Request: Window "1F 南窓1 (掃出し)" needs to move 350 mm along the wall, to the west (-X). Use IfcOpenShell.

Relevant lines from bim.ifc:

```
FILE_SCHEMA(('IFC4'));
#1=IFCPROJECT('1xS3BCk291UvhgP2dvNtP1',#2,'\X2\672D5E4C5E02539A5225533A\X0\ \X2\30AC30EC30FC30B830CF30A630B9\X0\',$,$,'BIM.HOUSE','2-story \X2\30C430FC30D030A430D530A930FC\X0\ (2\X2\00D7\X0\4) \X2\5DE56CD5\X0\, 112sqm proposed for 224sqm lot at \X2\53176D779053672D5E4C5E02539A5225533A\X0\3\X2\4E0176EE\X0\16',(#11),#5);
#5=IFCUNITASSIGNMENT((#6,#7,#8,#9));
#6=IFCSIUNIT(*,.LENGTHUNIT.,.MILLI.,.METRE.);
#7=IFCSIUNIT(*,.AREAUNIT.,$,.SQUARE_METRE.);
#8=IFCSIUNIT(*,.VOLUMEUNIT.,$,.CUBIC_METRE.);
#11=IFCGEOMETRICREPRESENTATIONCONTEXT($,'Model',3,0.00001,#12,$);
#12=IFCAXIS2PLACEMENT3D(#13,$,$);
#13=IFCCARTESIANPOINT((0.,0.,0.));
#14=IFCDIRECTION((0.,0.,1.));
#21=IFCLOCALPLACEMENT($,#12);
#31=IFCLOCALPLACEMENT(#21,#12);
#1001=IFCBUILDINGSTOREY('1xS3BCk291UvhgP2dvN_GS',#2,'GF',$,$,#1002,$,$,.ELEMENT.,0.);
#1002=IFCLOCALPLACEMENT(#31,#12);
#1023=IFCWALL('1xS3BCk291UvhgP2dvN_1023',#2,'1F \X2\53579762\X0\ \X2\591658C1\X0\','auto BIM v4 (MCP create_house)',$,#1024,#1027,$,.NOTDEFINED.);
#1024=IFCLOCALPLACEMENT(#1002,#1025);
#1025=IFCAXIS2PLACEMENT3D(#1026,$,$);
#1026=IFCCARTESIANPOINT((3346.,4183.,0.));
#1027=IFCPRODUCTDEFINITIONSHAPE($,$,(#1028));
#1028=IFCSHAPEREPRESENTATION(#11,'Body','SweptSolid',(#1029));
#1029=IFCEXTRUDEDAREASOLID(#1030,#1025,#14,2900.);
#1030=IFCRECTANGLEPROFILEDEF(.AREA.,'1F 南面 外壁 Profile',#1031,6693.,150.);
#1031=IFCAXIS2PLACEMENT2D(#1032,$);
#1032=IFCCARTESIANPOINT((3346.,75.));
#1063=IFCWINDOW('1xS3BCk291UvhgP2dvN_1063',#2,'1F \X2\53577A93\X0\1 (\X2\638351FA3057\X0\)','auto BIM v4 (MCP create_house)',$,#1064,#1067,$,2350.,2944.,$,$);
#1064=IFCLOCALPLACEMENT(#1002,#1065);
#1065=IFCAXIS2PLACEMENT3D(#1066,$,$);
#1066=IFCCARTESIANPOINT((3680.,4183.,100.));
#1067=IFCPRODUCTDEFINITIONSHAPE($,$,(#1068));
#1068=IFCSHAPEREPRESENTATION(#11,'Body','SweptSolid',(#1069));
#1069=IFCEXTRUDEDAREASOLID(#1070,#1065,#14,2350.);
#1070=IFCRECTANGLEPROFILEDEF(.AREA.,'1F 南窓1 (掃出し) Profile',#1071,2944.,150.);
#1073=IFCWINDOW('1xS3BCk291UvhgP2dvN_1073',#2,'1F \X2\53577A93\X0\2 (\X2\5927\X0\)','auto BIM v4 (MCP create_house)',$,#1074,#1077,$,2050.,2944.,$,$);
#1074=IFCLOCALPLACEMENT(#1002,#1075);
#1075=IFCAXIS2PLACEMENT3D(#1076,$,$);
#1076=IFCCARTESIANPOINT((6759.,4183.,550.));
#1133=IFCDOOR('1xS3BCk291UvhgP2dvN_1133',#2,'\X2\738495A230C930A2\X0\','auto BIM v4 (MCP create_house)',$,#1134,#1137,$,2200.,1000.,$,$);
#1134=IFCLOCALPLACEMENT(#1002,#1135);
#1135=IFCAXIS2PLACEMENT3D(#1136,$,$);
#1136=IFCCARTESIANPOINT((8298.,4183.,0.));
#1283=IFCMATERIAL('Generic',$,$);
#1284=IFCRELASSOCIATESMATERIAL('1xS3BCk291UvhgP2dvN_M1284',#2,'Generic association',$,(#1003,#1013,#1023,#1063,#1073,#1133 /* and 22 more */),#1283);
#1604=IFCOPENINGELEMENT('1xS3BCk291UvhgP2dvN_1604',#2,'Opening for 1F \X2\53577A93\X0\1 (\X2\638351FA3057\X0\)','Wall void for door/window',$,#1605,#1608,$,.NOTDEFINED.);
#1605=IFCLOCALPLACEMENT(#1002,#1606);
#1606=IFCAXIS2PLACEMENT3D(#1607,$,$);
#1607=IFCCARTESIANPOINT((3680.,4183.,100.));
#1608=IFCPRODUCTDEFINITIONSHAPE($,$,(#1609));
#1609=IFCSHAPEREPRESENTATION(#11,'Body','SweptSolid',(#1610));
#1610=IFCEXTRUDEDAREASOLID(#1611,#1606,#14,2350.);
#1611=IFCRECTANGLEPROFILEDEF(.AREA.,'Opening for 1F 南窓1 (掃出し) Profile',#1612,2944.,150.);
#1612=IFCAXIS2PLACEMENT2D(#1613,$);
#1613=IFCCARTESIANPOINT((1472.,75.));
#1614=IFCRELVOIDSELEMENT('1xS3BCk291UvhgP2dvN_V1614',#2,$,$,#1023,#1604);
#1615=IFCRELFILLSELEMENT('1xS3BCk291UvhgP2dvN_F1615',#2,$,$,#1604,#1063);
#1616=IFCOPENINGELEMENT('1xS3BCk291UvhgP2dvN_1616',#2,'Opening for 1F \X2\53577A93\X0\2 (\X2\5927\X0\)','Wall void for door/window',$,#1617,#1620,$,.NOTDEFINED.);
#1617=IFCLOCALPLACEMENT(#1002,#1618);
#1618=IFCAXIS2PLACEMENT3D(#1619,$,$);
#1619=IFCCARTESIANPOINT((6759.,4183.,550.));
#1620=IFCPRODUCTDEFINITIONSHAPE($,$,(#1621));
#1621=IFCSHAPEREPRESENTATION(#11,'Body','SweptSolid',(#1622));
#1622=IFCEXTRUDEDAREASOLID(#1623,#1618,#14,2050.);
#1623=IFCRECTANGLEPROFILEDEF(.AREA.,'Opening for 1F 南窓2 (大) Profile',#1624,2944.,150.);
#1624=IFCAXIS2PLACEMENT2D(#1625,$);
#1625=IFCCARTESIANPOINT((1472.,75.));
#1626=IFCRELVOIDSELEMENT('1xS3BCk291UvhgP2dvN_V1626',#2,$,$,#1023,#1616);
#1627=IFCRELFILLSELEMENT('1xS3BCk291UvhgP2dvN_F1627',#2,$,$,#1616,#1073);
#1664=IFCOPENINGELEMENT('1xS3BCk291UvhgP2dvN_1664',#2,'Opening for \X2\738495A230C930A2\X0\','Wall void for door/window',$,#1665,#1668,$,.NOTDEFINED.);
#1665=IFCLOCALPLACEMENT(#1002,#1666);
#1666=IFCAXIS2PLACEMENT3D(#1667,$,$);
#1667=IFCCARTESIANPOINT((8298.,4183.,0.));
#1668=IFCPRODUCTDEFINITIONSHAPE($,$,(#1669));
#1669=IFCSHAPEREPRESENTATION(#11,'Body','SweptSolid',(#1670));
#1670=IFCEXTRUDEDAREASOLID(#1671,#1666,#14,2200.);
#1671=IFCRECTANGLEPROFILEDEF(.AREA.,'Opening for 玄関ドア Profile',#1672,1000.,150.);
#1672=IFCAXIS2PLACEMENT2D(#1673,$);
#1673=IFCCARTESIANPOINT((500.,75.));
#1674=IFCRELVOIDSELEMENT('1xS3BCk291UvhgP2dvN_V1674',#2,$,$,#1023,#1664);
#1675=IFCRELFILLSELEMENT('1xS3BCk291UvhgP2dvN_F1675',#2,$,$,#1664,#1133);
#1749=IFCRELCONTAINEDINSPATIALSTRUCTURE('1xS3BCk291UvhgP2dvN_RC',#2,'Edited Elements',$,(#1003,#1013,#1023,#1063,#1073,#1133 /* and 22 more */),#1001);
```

```python
import ifcopenshell
import ifcopenshell.api.geometry
import ifcopenshell.util.placement
import ifcopenshell.util.unit

model = ifcopenshell.open("bim.ifc")
unit_scale = ifcopenshell.util.unit.calculate_unit_scale(model)

window = model.by_id(1063)
opening = window.FillsVoids[0].RelatingOpeningElement
wall = opening.VoidsElements[0].RelatingBuildingElement

wall_matrix = ifcopenshell.util.placement.get_local_placement(wall.ObjectPlacement)
shift = wall_matrix[:3, 0] * -0.35 / unit_scale
before = ifcopenshell.util.placement.get_local_placement(window.ObjectPlacement)[:3, 3].copy()

# The window is not placed relative to its opening, so move both.
for product in (opening, window):
    matrix = ifcopenshell.util.placement.get_local_placement(product.ObjectPlacement)
    matrix[:3, 3] += shift
    ifcopenshell.api.geometry.edit_object_placement(model, product=product, matrix=matrix, is_si=False)

after = ifcopenshell.util.placement.get_local_placement(window.ObjectPlacement)[:3, 3]
print("window moved by", (after - before).round(3) + 0.0)

model.write("bim_v2.ifc")
```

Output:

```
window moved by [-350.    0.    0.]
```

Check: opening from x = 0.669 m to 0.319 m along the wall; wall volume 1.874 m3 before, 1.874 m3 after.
